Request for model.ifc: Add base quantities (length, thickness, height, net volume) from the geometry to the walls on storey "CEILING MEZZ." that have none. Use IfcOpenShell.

First a look at what the model holds.

```python
import ifcopenshell
import ifcopenshell.util.element
import ifcopenshell.util.unit

model = ifcopenshell.open("model.ifc")
print(model.schema)
for unit_type in ("LENGTHUNIT", "AREAUNIT", "VOLUMEUNIT"):
    print(unit_type, ifcopenshell.util.unit.calculate_unit_scale(model, unit_type))
storey = next(s for s in model.by_type("IfcBuildingStorey") if s.Name == "CEILING MEZZ.")
walls = [e for e in ifcopenshell.util.element.get_decomposition(storey) if e.is_a("IfcWall")]
for e in sorted(walls, key=lambda e: e.id()):
    print(e.id(), e.is_a(), e.Name, list(ifcopenshell.util.element.get_psets(e, qtos_only=True)), sep=" | ")
```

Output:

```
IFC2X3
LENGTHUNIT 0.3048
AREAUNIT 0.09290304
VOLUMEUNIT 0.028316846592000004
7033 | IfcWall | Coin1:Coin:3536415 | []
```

```python
import ifcopenshell
import ifcopenshell.api.pset
import ifcopenshell.geom
import ifcopenshell.util.element
import ifcopenshell.util.shape
import ifcopenshell.util.unit

model = ifcopenshell.open("model.ifc")
unit_scale = ifcopenshell.util.unit.calculate_unit_scale(model)
volume_scale = ifcopenshell.util.unit.calculate_unit_scale(model, "VOLUMEUNIT")
settings = ifcopenshell.geom.settings()

storey = next(s for s in model.by_type("IfcBuildingStorey") if s.Name == "CEILING MEZZ.")
walls = [e for e in ifcopenshell.util.element.get_decomposition(storey) if e.is_a("IfcWall")]

for e in sorted(walls, key=lambda e: e.id()):
    if ifcopenshell.util.element.get_psets(e, qtos_only=True, should_inherit=False):
        continue
    # Geometry comes back in metres, in the element's own axes.
    shape = ifcopenshell.geom.create_shape(settings, e)
    values = {
        "Length": ifcopenshell.util.shape.get_x(shape.geometry) / unit_scale,
        "Width": ifcopenshell.util.shape.get_y(shape.geometry) / unit_scale,
        "Height": ifcopenshell.util.shape.get_z(shape.geometry) / unit_scale,
        "NetVolume": ifcopenshell.util.shape.get_volume(shape.geometry) / volume_scale,
    }
    qto = ifcopenshell.api.pset.add_qto(model, product=e, name="BaseQuantities")
    ifcopenshell.api.pset.edit_qto(model, qto=qto, properties=values)
    print(e.id(), {k: round(v, 3) for k, v in values.items()})

model.write("model_edited.ifc")
```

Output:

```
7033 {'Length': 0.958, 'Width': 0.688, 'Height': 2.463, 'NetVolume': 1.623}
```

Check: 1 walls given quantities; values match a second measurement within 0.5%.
